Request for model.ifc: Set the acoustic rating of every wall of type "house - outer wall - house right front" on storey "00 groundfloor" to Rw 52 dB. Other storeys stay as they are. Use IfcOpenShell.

First a look at what the model holds.

```python
import ifcopenshell
import ifcopenshell.util.element

model = ifcopenshell.open("model.ifc")
print(model.schema)
storey = next(s for s in model.by_type("IfcBuildingStorey") if s.Name == "00 groundfloor")
walls = [e for e in ifcopenshell.util.element.get_decomposition(storey) if e.is_a("IfcWall")]
seen = {}
for e in walls:
    element_type = ifcopenshell.util.element.get_type(e)
    key = (element_type.Name if element_type != e and element_type else None, ifcopenshell.util.element.get_pset(e, "Pset_WallCommon", "AcousticRating"))
    seen[key] = seen.get(key, 0) + 1
for (name, value), count in sorted(seen.items(), key=str):
    print(count, "x", name, "|", value)
```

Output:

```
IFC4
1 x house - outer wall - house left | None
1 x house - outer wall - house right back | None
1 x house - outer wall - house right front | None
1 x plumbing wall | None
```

```python
import ifcopenshell
import ifcopenshell.api.pset
import ifcopenshell.util.element

model = ifcopenshell.open("model.ifc")

storey = next(s for s in model.by_type("IfcBuildingStorey") if s.Name == "00 groundfloor")
walls = [e for e in ifcopenshell.util.element.get_decomposition(storey) if e.is_a("IfcWall")]

count = 0
for e in walls:
    element_type = ifcopenshell.util.element.get_type(e)
    if element_type in (None, e) or element_type.Name != "house - outer wall - house right front":
        continue
    # add_pset returns the element's existing set when there is one.
    pset = ifcopenshell.api.pset.add_pset(model, product=e, name="Pset_WallCommon")
    ifcopenshell.api.pset.edit_pset(model, pset=pset, properties={"AcousticRating": "Rw 52 dB"})
    count += 1

print(count, "walls updated")

model.write("model_edited.ifc")
```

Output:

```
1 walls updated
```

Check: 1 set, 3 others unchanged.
